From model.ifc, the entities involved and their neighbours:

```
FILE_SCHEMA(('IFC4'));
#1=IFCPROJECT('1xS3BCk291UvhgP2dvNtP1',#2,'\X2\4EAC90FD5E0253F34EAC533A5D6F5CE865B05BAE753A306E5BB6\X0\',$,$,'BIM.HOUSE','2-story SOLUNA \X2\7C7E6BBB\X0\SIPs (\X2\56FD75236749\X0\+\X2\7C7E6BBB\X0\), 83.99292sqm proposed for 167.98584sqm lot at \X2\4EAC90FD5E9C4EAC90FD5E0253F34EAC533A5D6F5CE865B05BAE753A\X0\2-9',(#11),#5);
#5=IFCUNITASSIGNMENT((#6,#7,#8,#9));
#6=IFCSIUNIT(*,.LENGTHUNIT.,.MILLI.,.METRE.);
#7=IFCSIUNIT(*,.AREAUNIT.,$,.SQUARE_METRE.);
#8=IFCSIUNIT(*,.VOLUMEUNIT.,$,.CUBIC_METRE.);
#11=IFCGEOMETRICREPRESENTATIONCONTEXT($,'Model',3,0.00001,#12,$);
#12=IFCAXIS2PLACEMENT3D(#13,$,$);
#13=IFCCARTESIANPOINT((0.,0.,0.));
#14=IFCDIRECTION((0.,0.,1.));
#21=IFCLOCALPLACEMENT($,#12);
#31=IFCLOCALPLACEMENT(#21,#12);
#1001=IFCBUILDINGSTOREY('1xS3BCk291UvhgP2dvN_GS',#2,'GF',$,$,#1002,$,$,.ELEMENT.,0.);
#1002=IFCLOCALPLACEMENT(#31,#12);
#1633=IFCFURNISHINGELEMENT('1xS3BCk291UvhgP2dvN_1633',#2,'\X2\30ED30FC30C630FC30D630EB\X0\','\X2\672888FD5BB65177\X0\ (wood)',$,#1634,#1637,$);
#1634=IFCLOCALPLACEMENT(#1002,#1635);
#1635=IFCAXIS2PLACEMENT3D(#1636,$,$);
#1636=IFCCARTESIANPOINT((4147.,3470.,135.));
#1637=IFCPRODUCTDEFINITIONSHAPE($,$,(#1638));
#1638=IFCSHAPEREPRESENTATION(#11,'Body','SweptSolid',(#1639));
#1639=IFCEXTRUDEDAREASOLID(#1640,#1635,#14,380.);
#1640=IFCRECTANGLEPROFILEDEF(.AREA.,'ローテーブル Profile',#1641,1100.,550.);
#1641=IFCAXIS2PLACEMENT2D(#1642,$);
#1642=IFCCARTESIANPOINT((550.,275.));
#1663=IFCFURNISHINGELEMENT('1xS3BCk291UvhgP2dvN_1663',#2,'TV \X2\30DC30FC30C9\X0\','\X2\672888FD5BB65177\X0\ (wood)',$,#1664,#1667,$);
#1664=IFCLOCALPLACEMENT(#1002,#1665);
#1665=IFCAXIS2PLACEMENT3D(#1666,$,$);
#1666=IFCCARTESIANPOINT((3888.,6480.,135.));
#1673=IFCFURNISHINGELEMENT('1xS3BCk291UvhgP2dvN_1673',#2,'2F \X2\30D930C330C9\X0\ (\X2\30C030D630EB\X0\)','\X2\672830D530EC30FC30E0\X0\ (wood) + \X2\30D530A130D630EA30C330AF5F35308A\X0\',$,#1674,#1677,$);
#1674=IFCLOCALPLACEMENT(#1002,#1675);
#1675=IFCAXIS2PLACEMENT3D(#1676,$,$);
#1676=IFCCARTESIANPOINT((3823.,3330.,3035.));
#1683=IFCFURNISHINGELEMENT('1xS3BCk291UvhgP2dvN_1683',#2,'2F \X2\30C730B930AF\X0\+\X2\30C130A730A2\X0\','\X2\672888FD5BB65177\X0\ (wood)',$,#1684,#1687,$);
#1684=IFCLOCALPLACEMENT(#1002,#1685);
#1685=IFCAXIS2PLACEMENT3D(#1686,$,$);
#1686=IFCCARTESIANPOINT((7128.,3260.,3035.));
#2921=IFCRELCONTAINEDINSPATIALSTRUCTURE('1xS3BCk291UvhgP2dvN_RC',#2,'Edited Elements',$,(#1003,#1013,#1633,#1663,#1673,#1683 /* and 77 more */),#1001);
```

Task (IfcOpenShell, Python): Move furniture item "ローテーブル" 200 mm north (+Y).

```python
import ifcopenshell
import ifcopenshell.api.geometry
import ifcopenshell.util.placement

model = ifcopenshell.open("model.ifc")

item = model.by_guid("1xS3BCk291UvhgP2dvN_1633")
matrix = ifcopenshell.util.placement.get_local_placement(item.ObjectPlacement)
matrix[1, 3] += 200.0
ifcopenshell.api.geometry.edit_object_placement(model, product=item, matrix=matrix, is_si=False)

print(ifcopenshell.util.placement.get_local_placement(item.ObjectPlacement).round(3) + 0.0)

model.write("model_v2.ifc")
```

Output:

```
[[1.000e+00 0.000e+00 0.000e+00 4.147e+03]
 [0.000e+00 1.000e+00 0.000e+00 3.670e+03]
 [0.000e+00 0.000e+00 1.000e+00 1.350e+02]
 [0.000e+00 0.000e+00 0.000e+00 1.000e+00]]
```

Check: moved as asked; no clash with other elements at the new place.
